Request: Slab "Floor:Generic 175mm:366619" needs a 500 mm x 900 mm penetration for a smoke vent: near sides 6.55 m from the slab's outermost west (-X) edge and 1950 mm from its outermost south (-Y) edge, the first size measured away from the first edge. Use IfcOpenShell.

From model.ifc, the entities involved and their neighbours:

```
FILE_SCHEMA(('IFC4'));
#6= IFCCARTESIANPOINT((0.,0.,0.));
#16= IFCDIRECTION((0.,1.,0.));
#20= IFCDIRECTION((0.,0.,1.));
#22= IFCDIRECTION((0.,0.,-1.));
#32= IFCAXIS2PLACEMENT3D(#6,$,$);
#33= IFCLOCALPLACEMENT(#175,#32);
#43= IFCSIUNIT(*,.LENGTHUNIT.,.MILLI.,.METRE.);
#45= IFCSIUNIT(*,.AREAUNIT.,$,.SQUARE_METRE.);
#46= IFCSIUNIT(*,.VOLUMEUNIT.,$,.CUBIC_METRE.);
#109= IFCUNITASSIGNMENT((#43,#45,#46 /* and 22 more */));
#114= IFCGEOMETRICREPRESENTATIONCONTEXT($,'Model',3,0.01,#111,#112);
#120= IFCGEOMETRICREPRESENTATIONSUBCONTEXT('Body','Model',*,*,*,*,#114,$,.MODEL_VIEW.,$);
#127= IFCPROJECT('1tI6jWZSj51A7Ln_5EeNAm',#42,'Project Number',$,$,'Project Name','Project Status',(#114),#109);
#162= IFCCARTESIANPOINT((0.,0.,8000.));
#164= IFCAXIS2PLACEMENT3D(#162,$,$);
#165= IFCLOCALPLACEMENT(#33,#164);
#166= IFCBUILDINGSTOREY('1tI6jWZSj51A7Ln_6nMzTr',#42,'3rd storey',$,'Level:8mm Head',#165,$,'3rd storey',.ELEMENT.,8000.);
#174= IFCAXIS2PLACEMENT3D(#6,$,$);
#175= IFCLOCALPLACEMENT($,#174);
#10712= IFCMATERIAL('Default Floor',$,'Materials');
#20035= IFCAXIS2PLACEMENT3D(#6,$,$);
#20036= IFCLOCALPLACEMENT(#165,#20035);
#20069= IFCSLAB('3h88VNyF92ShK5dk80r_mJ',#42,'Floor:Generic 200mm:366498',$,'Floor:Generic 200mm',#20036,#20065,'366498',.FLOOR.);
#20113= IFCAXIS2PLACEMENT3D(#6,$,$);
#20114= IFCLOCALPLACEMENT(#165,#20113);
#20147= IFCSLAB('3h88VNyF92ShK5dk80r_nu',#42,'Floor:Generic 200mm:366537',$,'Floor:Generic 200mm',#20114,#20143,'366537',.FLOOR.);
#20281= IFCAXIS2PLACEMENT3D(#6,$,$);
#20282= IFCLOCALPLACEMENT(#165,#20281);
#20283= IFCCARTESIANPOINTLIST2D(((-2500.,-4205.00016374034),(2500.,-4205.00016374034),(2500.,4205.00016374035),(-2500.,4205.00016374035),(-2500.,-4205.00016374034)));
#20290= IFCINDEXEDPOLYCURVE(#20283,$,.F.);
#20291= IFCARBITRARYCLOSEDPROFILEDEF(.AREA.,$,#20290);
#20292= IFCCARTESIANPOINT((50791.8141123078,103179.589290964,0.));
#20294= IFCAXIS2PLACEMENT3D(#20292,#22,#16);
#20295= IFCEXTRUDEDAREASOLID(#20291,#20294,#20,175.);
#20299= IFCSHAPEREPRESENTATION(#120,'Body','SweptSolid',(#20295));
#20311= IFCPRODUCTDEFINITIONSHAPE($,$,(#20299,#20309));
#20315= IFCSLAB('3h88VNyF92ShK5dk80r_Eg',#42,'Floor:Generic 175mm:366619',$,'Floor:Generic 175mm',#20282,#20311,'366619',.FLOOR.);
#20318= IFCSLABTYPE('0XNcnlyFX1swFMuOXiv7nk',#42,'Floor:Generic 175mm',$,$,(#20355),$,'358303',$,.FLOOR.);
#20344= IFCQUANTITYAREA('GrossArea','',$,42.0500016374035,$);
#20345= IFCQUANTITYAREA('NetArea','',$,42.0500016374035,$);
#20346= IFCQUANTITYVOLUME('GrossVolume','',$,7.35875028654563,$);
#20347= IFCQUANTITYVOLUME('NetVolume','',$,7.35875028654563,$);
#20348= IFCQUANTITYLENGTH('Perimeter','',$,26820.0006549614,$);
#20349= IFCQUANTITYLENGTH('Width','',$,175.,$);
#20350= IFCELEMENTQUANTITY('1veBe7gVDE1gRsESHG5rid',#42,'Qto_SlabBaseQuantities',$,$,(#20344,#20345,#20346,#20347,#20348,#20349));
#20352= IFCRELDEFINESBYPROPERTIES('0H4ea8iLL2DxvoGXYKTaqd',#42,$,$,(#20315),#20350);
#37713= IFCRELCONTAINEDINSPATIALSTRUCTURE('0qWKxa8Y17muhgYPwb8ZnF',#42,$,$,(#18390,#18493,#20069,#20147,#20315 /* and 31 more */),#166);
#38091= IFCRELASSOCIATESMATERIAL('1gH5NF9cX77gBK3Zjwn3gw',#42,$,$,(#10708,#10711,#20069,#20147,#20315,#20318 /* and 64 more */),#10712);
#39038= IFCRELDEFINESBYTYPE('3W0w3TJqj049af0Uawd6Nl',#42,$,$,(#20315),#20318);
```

```python
import numpy as np
import ifcopenshell
import ifcopenshell.api.feature
import ifcopenshell.api.geometry
import ifcopenshell.api.pset
import ifcopenshell.api.root
import ifcopenshell.geom
import ifcopenshell.util.element
import ifcopenshell.util.placement
import ifcopenshell.util.representation
import ifcopenshell.util.shape
import ifcopenshell.util.unit

model = ifcopenshell.open("model.ifc")
unit_scale = ifcopenshell.util.unit.calculate_unit_scale(model)
area_scale = ifcopenshell.util.unit.calculate_unit_scale(model, "AREAUNIT")
volume_scale = ifcopenshell.util.unit.calculate_unit_scale(model, "VOLUMEUNIT")
settings = ifcopenshell.geom.settings()


def volume(element):
    """Net volume in cubic metres, openings subtracted."""
    shape = ifcopenshell.geom.create_shape(settings, element)
    return ifcopenshell.util.shape.get_volume(shape.geometry)


slab = model.by_guid("3h88VNyF92ShK5dk80r_Eg")
before = volume(slab)

# Extent in the slab's own axes, in metres. The edges named are its -X and -Y sides.
slab_shape = ifcopenshell.geom.create_shape(settings, slab)
vertices = ifcopenshell.util.shape.get_vertices(slab_shape.geometry)
x_min, y_min, bottom = vertices.min(axis=0)
top = vertices[:, 2].max()

opening = ifcopenshell.api.root.create_entity(model, ifc_class="IfcOpeningElement", name="Smoke vent opening", predefined_type="OPENING")
context = ifcopenshell.util.representation.get_context(model, "Model", "Body", "MODEL_VIEW")
width, depth = 0.5, 0.9
outline = [(0.0, 0.0), (width, 0.0), (width, depth), (0.0, depth), (0.0, 0.0)]
# Overshoot both faces by 50 mm so the cut is clean.
shape = ifcopenshell.api.geometry.add_slab_representation(
    model, context=context, depth=top - bottom + 0.1, polyline=outline
)
ifcopenshell.api.geometry.assign_representation(model, product=opening, representation=shape)

matrix = ifcopenshell.util.placement.get_local_placement(slab.ObjectPlacement)
matrix[:, 3] = matrix @ np.append(np.array([x_min + 6.55, y_min + 1.95, bottom - 0.05]) / unit_scale, 1.0)
ifcopenshell.api.geometry.edit_object_placement(model, product=opening, matrix=matrix, is_si=False)
ifcopenshell.api.feature.add_feature(model, feature=opening, element=slab)

after = volume(slab)

# Update the slab's stored quantities.
qto = model.by_id(ifcopenshell.util.element.get_pset(slab, "Qto_SlabBaseQuantities", should_inherit=False)["id"])
ifcopenshell.api.pset.edit_qto(model, qto=qto, properties={
    "NetArea": after / (top - bottom) / area_scale,
    "NetVolume": after / volume_scale,
})

print(f"slab volume {before:.3f} -> {after:.3f} m3")

model.write("model_edited.ifc")
```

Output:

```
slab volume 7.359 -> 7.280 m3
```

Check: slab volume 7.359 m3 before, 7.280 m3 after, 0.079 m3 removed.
